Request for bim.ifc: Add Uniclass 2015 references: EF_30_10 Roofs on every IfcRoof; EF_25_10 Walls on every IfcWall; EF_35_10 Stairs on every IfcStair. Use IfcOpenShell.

First a look at what the model holds.

```python
import ifcopenshell

model = ifcopenshell.open("bim.ifc")
print(model.schema)
print("classifications:", [c.Name for c in model.by_type("IfcClassification")])
for ifc_class in ("IfcDoor", "IfcRoof", "IfcStair", "IfcWall", "IfcWindow"):
    print(ifc_class, len(model.by_type(ifc_class)))
```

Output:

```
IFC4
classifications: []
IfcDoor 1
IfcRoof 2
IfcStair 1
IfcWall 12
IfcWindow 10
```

```python
import ifcopenshell
import ifcopenshell.api.classification

model = ifcopenshell.open("bim.ifc")

system = ifcopenshell.api.classification.add_classification(model, classification="Uniclass 2015")

codes = {
    "IfcRoof": ("EF_30_10", "Roofs"),
    "IfcWall": ("EF_25_10", "Walls"),
    "IfcStair": ("EF_35_10", "Stairs"),
}
for ifc_class, (code, name) in codes.items():
    products = model.by_type(ifc_class)
    ifcopenshell.api.classification.add_reference(
        model, products=products, classification=system, identification=code, name=name
    )
    print(code, len(products))

model.write("bim_v2.ifc")
```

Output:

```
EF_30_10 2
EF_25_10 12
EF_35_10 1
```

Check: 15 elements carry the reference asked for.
